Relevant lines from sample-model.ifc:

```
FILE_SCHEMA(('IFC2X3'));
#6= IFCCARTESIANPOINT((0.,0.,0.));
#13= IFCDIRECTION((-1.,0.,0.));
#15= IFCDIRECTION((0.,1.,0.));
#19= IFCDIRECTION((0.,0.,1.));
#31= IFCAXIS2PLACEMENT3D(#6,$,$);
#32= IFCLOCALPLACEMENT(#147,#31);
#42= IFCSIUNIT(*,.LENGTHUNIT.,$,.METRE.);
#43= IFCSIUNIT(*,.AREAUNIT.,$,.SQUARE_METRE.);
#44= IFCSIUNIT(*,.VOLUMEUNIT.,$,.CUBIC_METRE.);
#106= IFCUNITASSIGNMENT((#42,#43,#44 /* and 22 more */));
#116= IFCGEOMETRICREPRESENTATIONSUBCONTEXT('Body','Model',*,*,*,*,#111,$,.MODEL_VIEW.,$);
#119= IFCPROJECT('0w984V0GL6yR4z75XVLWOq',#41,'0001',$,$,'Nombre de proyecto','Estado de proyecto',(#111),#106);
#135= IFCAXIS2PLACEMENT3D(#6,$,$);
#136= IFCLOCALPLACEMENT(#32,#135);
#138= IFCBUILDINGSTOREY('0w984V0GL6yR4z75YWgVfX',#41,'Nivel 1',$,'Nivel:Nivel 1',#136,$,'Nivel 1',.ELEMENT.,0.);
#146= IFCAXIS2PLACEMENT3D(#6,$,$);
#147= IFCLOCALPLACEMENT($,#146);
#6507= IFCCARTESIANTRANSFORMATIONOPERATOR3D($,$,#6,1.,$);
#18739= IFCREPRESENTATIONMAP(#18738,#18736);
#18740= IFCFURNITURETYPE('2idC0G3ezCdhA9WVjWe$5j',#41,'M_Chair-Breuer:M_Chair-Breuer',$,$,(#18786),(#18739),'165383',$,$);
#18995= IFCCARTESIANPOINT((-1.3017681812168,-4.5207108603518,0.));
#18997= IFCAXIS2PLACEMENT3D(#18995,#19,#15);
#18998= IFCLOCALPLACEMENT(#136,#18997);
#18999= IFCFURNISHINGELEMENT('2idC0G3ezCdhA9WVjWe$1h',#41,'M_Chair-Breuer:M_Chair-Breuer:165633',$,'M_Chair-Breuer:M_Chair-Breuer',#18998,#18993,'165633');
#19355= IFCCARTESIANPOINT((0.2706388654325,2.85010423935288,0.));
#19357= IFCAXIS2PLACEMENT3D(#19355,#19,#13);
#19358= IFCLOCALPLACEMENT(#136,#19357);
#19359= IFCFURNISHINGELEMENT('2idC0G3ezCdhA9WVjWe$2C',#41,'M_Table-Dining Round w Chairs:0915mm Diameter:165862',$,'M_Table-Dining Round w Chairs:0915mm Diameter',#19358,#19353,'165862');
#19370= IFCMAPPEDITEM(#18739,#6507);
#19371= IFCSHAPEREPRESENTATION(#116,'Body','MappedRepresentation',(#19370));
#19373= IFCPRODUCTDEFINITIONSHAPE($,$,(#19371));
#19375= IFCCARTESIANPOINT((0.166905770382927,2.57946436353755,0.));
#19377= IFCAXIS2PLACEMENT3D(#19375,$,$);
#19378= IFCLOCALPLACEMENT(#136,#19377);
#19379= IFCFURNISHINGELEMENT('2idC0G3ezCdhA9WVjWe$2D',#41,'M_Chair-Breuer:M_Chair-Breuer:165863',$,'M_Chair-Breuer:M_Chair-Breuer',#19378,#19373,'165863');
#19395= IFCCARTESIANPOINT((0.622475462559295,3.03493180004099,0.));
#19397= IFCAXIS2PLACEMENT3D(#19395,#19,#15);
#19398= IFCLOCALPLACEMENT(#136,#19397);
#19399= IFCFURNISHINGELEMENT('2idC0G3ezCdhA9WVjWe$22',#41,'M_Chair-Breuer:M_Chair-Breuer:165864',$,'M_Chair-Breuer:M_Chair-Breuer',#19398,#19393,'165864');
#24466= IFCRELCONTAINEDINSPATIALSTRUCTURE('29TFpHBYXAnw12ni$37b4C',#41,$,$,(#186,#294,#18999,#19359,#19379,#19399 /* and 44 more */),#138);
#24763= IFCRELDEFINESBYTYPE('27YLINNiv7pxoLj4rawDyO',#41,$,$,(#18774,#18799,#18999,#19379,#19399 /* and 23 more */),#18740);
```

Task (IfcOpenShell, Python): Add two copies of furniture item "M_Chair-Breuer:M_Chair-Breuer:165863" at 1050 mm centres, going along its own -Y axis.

```python
import ifcopenshell
import ifcopenshell.api.geometry
import ifcopenshell.api.root
import ifcopenshell.util.element
import ifcopenshell.util.placement
import ifcopenshell.util.unit

model = ifcopenshell.open("sample-model.ifc")
unit_scale = ifcopenshell.util.unit.calculate_unit_scale(model)


def reuse_history(source, copy):
    """copy_class also copies each property set's owner history, people and application; keep the originals."""
    for rel in copy.IsDefinedBy:
        if rel.is_a("IfcRelDefinesByProperties") and (history := rel.RelatingPropertyDefinition.OwnerHistory):
            rel.RelatingPropertyDefinition.OwnerHistory = source.OwnerHistory
            ifcopenshell.util.element.remove_deep2(model, history)


source = model.by_guid("2idC0G3ezCdhA9WVjWe$2D")
base = ifcopenshell.util.placement.get_local_placement(source.ObjectPlacement)
step = -base[:3, 1] * 1.05 / unit_scale

for i in range(1, 3):
    copy = ifcopenshell.api.root.copy_class(model, product=source)
    copy.Representation = ifcopenshell.util.element.copy_deep(
        model, source.Representation, exclude=["IfcGeometricRepresentationContext", "IfcRepresentationMap"]
    )
    copy.Name = "M_Chair-Breuer:M_Chair-Breuer"
    copy.Tag = None
    reuse_history(source, copy)
    matrix = base.copy()
    matrix[:3, 3] += i * step
    print("added at", matrix[:3, 3].round(3) + 0.0)
    ifcopenshell.api.geometry.edit_object_placement(model, product=copy, matrix=matrix, is_si=False)

model.write("sample-model_v2.ifc")
```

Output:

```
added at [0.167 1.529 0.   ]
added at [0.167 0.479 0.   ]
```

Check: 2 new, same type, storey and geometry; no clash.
